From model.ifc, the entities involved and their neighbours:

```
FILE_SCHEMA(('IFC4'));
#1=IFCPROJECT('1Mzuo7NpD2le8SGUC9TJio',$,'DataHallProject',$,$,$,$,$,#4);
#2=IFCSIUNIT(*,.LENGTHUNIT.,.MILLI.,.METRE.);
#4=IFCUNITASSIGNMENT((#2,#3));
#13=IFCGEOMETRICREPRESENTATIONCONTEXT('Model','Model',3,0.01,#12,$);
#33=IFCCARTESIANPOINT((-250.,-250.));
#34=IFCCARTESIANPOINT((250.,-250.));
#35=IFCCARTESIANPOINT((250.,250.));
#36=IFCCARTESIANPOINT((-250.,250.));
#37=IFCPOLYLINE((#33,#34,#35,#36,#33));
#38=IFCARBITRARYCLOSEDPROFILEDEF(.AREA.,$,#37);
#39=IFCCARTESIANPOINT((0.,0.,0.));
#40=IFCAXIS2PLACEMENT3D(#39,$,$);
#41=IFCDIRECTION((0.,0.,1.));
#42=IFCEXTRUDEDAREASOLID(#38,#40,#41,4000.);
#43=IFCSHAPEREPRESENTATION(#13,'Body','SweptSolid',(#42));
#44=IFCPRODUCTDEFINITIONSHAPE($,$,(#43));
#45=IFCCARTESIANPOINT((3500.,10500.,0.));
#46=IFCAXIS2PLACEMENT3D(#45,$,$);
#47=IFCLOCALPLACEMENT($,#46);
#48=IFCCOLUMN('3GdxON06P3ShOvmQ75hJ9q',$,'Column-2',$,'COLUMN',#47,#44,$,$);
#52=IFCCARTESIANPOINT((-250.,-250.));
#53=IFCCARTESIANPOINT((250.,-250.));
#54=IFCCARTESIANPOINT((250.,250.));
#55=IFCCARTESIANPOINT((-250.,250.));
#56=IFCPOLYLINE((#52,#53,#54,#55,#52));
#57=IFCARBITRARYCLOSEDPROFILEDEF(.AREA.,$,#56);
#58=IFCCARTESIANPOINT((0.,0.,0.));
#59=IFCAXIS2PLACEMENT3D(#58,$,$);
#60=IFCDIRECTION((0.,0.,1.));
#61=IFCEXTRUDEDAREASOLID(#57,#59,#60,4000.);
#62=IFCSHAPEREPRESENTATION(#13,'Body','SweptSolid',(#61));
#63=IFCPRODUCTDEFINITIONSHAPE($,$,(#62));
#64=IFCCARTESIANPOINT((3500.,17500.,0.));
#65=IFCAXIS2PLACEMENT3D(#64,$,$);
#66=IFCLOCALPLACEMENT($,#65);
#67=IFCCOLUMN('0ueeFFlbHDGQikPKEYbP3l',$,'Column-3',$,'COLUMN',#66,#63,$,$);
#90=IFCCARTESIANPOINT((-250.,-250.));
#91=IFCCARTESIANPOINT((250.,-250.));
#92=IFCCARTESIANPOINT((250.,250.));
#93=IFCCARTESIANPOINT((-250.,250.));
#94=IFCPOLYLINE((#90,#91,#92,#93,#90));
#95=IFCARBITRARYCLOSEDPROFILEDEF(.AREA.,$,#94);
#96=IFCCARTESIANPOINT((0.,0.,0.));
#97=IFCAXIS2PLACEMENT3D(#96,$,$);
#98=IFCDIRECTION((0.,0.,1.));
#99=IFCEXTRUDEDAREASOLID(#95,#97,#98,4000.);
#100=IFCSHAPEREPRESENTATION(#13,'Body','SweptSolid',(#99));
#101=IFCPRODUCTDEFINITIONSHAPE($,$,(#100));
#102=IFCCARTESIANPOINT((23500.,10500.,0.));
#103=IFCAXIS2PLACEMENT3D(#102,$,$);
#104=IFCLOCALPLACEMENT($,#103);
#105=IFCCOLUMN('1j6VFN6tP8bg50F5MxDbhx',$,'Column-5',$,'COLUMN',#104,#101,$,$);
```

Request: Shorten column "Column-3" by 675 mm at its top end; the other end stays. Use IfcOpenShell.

```python
import ifcopenshell
import ifcopenshell.util.unit

model = ifcopenshell.open("model.ifc")
unit_scale = ifcopenshell.util.unit.calculate_unit_scale(model)

member = model.by_guid("0ueeFFlbHDGQikPKEYbP3l")
change = -0.675 / unit_scale

# The extrusion runs towards the end named, so only its depth changes.
body = next(r for r in member.Representation.Representations if r.RepresentationIdentifier == "Body")
solid = body.Items[0]
old_length = solid.Depth
solid.Depth += change

print(f"length {old_length:g} -> {solid.Depth:g}")

model.write("model_rev.ifc")
```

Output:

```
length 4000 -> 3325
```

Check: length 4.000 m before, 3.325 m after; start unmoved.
